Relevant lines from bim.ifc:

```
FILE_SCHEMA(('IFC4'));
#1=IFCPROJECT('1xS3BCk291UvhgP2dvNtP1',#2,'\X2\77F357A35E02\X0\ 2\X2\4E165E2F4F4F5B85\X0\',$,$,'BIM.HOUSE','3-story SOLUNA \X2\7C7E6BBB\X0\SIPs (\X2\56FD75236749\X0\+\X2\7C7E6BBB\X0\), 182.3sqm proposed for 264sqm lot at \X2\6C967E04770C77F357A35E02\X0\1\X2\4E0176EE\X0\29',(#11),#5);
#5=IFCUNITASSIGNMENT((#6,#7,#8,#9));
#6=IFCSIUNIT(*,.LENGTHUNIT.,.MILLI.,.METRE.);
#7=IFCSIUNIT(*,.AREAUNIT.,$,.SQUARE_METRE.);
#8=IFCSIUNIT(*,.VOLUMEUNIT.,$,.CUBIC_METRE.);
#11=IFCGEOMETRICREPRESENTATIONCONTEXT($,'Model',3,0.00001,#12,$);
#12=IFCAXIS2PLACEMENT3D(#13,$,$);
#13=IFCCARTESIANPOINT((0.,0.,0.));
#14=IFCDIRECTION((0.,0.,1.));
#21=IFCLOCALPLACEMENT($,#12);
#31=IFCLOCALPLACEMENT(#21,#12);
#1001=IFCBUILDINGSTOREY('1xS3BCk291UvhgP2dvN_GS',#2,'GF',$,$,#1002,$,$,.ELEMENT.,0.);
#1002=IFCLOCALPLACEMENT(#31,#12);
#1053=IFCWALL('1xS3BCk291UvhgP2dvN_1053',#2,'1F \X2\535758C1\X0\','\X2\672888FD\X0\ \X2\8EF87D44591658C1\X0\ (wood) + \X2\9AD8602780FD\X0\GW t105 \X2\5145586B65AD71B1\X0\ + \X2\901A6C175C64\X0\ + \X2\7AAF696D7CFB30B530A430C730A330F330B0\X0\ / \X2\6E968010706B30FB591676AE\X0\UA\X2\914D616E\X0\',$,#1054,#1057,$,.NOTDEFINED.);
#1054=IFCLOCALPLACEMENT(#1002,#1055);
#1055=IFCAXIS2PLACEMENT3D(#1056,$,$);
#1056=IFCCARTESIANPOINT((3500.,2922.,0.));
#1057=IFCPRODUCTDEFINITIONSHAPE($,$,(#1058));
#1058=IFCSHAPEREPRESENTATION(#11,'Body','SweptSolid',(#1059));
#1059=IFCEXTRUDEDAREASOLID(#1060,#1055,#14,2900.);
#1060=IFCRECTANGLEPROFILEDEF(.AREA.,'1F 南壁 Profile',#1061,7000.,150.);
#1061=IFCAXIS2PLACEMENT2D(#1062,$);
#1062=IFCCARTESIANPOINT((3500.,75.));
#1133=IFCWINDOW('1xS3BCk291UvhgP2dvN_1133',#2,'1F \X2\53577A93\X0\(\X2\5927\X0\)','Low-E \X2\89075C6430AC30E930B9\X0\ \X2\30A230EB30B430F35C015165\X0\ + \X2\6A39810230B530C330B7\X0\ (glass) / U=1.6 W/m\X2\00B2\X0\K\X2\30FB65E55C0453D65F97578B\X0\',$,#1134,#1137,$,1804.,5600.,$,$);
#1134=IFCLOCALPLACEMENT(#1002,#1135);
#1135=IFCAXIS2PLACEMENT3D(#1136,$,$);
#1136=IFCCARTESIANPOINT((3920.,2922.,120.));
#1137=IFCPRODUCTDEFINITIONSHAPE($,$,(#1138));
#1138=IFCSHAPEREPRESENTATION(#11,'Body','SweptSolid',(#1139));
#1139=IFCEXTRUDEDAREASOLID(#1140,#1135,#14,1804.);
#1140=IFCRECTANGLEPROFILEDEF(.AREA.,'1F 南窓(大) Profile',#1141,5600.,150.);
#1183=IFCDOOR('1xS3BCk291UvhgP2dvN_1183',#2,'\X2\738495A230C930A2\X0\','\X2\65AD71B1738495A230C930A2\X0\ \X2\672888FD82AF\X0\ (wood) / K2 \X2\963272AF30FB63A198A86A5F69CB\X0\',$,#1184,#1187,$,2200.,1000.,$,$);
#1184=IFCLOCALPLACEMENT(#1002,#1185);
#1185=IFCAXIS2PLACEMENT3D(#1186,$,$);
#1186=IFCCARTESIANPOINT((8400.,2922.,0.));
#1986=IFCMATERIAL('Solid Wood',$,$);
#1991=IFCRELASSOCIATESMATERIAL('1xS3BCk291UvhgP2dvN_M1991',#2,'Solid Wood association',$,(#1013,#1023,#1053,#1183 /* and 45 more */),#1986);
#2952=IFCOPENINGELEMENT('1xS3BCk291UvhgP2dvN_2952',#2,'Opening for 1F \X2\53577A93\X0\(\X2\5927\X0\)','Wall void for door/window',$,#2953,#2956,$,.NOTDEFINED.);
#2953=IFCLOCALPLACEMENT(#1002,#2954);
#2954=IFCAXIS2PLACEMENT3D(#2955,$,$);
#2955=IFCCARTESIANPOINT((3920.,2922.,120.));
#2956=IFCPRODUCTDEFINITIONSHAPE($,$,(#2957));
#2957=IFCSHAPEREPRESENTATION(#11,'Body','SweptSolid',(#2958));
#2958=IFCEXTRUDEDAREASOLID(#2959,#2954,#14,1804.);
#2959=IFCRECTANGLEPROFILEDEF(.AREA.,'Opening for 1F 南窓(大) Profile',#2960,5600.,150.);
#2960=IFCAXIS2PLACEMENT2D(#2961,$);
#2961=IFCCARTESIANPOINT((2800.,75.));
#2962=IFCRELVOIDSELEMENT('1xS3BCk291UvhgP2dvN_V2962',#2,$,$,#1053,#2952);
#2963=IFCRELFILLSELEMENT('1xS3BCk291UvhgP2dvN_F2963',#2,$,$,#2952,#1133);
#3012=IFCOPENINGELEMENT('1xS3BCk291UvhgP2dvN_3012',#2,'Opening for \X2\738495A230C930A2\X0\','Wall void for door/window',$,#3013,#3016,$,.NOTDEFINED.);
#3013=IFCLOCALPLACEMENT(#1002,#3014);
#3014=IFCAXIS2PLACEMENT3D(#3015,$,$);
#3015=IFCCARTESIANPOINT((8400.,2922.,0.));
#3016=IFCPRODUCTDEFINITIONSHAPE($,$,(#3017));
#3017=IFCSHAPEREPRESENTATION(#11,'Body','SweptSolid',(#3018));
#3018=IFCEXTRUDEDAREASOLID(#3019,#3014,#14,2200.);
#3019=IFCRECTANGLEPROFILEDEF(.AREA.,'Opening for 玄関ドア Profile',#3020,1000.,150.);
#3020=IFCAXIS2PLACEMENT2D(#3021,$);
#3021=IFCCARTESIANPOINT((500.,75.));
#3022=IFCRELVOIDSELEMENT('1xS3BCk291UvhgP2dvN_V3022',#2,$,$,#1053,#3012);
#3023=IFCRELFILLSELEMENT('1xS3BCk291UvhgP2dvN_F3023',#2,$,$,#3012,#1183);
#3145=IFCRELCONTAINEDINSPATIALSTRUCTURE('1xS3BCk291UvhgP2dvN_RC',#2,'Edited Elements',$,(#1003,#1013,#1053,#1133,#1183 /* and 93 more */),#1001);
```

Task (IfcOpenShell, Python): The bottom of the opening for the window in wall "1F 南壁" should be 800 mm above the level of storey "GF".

```python
import numpy as np
import ifcopenshell
import ifcopenshell.api.geometry
import ifcopenshell.geom
import ifcopenshell.util.element
import ifcopenshell.util.placement
import ifcopenshell.util.shape
import ifcopenshell.util.unit

model = ifcopenshell.open("bim.ifc")
unit_scale = ifcopenshell.util.unit.calculate_unit_scale(model)

window = model.by_guid("1xS3BCk291UvhgP2dvN_1133")
opening = window.FillsVoids[0].RelatingOpeningElement
storey = ifcopenshell.util.element.get_container(window, ifc_class="IfcBuildingStorey")
level = ifcopenshell.util.placement.get_local_placement(storey.ObjectPlacement)[2, 3]

# The opening's origin need not be at the sill, so measure its lowest point.
shape = ifcopenshell.geom.create_shape(ifcopenshell.geom.settings(), opening)
bottom = ifcopenshell.util.shape.get_shape_bottom_elevation(shape, shape.geometry) / unit_scale
dz = level + 0.8 / unit_scale - bottom

shift = np.array([0.0, 0.0, dz])
# The window is not placed relative to its opening, so move both.
for product in (opening, window):
    matrix = ifcopenshell.util.placement.get_local_placement(product.ObjectPlacement)
    matrix[:3, 3] += shift
    ifcopenshell.api.geometry.edit_object_placement(model, product=product, matrix=matrix, is_si=False)

print(f"moved by {dz * unit_scale:+.3f} m")

model.write("bim_rev.ifc")
```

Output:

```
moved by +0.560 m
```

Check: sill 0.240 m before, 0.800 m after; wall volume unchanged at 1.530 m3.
